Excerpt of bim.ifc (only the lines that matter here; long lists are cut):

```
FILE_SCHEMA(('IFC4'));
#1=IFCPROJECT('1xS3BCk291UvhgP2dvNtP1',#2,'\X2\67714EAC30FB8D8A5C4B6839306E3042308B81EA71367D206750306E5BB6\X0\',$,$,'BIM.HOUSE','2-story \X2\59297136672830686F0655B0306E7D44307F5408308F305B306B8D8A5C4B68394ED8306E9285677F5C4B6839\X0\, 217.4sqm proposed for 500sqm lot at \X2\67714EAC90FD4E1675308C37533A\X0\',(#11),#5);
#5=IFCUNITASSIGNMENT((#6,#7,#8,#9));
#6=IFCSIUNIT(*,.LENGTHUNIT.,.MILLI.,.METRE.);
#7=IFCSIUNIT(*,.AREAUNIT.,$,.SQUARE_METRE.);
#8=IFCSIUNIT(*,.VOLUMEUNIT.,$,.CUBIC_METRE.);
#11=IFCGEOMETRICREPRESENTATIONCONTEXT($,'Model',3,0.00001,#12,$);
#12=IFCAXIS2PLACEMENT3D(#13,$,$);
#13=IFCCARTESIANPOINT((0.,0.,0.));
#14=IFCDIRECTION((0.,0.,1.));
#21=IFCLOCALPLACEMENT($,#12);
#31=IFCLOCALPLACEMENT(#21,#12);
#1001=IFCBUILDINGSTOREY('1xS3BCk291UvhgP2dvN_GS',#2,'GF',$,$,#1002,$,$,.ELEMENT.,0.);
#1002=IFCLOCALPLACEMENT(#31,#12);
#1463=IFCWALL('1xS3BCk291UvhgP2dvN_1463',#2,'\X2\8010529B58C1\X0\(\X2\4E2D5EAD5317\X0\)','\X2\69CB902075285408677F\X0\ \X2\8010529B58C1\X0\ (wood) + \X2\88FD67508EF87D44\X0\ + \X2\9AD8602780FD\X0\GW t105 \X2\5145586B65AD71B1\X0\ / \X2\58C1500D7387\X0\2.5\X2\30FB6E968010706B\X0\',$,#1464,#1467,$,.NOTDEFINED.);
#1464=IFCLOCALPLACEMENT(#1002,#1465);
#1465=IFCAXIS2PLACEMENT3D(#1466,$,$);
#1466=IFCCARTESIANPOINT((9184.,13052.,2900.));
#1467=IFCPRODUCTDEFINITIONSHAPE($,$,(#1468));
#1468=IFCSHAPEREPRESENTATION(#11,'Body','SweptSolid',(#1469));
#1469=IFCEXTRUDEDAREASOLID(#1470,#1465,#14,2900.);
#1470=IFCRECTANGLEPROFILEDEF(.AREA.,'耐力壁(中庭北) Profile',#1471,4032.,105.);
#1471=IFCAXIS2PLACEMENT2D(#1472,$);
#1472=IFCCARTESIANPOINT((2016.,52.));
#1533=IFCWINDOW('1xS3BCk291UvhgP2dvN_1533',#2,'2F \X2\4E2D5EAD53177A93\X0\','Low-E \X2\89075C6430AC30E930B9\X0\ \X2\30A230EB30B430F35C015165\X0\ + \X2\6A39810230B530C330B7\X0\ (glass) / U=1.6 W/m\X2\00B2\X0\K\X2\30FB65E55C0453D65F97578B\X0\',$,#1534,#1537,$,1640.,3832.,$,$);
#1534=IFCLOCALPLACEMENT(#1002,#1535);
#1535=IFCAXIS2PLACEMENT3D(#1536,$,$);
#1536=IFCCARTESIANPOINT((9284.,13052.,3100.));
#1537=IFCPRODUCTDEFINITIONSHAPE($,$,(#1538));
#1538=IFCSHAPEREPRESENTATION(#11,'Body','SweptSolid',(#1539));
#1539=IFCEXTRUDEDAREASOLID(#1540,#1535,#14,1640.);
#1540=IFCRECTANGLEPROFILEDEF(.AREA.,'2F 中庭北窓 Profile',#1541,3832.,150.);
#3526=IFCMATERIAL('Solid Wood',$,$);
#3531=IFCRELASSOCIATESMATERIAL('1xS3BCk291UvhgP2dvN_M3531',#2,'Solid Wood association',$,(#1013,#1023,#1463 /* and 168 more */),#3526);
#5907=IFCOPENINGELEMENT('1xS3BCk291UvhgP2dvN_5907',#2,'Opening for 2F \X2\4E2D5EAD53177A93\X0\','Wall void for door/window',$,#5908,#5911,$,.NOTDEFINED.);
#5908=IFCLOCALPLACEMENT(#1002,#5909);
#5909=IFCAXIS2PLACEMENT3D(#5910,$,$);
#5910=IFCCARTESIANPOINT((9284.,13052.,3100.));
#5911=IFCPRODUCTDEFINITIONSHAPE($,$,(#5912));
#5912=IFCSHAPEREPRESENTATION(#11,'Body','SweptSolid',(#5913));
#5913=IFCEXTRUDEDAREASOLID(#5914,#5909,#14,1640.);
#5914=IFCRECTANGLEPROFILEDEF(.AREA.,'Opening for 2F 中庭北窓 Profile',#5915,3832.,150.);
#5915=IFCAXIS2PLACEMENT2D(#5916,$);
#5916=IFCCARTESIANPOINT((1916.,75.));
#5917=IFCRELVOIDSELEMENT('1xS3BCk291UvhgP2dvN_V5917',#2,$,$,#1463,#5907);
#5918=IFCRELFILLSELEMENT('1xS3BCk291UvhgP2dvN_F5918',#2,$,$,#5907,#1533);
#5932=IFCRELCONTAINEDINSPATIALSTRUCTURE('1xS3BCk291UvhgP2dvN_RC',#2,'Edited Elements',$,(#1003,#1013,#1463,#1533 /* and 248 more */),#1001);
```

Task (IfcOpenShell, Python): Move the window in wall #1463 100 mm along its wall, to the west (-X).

```python
import ifcopenshell
import ifcopenshell.api.geometry
import ifcopenshell.util.placement
import ifcopenshell.util.unit

model = ifcopenshell.open("bim.ifc")
unit_scale = ifcopenshell.util.unit.calculate_unit_scale(model)

window = model.by_guid("1xS3BCk291UvhgP2dvN_1533")
opening = window.FillsVoids[0].RelatingOpeningElement
wall = opening.VoidsElements[0].RelatingBuildingElement

wall_matrix = ifcopenshell.util.placement.get_local_placement(wall.ObjectPlacement)
shift = wall_matrix[:3, 0] * -0.1 / unit_scale
before = ifcopenshell.util.placement.get_local_placement(window.ObjectPlacement)[:3, 3].copy()

# The window is not placed relative to its opening, so move both.
for product in (opening, window):
    matrix = ifcopenshell.util.placement.get_local_placement(product.ObjectPlacement)
    matrix[:3, 3] += shift
    ifcopenshell.api.geometry.edit_object_placement(model, product=product, matrix=matrix, is_si=False)

after = ifcopenshell.util.placement.get_local_placement(window.ObjectPlacement)[:3, 3]
print("window moved by", (after - before).round(3) + 0.0)

model.write("bim-out.ifc")
```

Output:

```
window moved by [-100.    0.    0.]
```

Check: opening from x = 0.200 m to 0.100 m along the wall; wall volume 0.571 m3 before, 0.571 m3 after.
